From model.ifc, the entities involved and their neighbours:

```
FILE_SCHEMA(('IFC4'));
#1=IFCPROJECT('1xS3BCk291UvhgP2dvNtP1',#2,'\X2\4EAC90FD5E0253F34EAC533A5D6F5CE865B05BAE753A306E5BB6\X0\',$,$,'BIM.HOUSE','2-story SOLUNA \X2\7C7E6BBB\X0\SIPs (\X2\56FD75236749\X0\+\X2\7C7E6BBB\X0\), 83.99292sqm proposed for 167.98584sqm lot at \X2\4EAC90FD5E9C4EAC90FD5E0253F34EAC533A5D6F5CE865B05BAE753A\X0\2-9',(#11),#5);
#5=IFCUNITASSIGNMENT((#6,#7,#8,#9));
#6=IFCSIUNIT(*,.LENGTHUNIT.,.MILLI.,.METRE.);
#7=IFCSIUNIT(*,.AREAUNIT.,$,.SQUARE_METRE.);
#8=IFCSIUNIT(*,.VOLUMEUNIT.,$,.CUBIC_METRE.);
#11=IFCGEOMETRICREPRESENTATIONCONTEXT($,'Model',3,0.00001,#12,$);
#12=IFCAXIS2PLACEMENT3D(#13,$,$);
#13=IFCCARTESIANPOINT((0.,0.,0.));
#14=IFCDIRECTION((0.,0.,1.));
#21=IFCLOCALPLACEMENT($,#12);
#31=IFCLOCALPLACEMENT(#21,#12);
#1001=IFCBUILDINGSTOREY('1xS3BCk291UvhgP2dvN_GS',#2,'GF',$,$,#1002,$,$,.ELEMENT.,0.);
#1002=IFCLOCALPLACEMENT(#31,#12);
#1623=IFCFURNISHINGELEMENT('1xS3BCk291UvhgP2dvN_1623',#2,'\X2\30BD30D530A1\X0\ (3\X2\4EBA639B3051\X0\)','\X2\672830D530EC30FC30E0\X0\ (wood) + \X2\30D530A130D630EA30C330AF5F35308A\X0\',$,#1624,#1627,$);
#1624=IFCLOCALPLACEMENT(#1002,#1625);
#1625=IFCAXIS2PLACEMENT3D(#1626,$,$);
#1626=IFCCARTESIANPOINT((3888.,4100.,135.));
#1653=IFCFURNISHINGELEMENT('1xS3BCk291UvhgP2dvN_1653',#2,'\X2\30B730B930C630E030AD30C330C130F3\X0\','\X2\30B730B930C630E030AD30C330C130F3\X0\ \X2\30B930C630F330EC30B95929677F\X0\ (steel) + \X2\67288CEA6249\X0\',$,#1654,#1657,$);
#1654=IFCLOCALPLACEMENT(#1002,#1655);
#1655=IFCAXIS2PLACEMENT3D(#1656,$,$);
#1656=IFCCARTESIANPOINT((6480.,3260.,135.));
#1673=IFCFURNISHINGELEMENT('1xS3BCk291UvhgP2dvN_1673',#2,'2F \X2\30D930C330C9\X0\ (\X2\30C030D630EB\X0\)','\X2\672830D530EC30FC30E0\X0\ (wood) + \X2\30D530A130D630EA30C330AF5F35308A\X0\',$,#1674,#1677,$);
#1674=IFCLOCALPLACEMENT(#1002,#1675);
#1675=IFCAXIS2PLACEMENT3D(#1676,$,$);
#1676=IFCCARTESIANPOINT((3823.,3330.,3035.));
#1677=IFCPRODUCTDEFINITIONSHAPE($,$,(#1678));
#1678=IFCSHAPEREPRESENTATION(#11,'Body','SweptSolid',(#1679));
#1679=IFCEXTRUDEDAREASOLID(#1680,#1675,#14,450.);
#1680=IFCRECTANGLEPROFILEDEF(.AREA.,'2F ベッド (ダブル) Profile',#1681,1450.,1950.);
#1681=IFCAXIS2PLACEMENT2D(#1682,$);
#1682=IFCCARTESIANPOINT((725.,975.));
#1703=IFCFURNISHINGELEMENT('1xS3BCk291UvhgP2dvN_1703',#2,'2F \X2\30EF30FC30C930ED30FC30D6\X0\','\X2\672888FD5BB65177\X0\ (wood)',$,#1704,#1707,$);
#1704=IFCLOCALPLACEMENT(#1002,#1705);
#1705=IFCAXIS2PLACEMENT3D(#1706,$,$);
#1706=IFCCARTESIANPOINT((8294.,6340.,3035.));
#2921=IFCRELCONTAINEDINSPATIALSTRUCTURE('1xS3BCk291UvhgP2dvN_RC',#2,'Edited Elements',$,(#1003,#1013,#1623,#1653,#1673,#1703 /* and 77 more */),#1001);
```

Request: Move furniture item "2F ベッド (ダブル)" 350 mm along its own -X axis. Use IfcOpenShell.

```python
import ifcopenshell
import ifcopenshell.api.geometry
import ifcopenshell.util.placement
import ifcopenshell.util.unit

model = ifcopenshell.open("model.ifc")
unit_scale = ifcopenshell.util.unit.calculate_unit_scale(model)

item = model.by_guid("1xS3BCk291UvhgP2dvN_1673")
matrix = ifcopenshell.util.placement.get_local_placement(item.ObjectPlacement)
matrix[:3, 3] -= matrix[:3, 0] * 0.35 / unit_scale
ifcopenshell.api.geometry.edit_object_placement(model, product=item, matrix=matrix, is_si=False)

print(ifcopenshell.util.placement.get_local_placement(item.ObjectPlacement).round(3) + 0.0)

model.write("model_updated.ifc")
```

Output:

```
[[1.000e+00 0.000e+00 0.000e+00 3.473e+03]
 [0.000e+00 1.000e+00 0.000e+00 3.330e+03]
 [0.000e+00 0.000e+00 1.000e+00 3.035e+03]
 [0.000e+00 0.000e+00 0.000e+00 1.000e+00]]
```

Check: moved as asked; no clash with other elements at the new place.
